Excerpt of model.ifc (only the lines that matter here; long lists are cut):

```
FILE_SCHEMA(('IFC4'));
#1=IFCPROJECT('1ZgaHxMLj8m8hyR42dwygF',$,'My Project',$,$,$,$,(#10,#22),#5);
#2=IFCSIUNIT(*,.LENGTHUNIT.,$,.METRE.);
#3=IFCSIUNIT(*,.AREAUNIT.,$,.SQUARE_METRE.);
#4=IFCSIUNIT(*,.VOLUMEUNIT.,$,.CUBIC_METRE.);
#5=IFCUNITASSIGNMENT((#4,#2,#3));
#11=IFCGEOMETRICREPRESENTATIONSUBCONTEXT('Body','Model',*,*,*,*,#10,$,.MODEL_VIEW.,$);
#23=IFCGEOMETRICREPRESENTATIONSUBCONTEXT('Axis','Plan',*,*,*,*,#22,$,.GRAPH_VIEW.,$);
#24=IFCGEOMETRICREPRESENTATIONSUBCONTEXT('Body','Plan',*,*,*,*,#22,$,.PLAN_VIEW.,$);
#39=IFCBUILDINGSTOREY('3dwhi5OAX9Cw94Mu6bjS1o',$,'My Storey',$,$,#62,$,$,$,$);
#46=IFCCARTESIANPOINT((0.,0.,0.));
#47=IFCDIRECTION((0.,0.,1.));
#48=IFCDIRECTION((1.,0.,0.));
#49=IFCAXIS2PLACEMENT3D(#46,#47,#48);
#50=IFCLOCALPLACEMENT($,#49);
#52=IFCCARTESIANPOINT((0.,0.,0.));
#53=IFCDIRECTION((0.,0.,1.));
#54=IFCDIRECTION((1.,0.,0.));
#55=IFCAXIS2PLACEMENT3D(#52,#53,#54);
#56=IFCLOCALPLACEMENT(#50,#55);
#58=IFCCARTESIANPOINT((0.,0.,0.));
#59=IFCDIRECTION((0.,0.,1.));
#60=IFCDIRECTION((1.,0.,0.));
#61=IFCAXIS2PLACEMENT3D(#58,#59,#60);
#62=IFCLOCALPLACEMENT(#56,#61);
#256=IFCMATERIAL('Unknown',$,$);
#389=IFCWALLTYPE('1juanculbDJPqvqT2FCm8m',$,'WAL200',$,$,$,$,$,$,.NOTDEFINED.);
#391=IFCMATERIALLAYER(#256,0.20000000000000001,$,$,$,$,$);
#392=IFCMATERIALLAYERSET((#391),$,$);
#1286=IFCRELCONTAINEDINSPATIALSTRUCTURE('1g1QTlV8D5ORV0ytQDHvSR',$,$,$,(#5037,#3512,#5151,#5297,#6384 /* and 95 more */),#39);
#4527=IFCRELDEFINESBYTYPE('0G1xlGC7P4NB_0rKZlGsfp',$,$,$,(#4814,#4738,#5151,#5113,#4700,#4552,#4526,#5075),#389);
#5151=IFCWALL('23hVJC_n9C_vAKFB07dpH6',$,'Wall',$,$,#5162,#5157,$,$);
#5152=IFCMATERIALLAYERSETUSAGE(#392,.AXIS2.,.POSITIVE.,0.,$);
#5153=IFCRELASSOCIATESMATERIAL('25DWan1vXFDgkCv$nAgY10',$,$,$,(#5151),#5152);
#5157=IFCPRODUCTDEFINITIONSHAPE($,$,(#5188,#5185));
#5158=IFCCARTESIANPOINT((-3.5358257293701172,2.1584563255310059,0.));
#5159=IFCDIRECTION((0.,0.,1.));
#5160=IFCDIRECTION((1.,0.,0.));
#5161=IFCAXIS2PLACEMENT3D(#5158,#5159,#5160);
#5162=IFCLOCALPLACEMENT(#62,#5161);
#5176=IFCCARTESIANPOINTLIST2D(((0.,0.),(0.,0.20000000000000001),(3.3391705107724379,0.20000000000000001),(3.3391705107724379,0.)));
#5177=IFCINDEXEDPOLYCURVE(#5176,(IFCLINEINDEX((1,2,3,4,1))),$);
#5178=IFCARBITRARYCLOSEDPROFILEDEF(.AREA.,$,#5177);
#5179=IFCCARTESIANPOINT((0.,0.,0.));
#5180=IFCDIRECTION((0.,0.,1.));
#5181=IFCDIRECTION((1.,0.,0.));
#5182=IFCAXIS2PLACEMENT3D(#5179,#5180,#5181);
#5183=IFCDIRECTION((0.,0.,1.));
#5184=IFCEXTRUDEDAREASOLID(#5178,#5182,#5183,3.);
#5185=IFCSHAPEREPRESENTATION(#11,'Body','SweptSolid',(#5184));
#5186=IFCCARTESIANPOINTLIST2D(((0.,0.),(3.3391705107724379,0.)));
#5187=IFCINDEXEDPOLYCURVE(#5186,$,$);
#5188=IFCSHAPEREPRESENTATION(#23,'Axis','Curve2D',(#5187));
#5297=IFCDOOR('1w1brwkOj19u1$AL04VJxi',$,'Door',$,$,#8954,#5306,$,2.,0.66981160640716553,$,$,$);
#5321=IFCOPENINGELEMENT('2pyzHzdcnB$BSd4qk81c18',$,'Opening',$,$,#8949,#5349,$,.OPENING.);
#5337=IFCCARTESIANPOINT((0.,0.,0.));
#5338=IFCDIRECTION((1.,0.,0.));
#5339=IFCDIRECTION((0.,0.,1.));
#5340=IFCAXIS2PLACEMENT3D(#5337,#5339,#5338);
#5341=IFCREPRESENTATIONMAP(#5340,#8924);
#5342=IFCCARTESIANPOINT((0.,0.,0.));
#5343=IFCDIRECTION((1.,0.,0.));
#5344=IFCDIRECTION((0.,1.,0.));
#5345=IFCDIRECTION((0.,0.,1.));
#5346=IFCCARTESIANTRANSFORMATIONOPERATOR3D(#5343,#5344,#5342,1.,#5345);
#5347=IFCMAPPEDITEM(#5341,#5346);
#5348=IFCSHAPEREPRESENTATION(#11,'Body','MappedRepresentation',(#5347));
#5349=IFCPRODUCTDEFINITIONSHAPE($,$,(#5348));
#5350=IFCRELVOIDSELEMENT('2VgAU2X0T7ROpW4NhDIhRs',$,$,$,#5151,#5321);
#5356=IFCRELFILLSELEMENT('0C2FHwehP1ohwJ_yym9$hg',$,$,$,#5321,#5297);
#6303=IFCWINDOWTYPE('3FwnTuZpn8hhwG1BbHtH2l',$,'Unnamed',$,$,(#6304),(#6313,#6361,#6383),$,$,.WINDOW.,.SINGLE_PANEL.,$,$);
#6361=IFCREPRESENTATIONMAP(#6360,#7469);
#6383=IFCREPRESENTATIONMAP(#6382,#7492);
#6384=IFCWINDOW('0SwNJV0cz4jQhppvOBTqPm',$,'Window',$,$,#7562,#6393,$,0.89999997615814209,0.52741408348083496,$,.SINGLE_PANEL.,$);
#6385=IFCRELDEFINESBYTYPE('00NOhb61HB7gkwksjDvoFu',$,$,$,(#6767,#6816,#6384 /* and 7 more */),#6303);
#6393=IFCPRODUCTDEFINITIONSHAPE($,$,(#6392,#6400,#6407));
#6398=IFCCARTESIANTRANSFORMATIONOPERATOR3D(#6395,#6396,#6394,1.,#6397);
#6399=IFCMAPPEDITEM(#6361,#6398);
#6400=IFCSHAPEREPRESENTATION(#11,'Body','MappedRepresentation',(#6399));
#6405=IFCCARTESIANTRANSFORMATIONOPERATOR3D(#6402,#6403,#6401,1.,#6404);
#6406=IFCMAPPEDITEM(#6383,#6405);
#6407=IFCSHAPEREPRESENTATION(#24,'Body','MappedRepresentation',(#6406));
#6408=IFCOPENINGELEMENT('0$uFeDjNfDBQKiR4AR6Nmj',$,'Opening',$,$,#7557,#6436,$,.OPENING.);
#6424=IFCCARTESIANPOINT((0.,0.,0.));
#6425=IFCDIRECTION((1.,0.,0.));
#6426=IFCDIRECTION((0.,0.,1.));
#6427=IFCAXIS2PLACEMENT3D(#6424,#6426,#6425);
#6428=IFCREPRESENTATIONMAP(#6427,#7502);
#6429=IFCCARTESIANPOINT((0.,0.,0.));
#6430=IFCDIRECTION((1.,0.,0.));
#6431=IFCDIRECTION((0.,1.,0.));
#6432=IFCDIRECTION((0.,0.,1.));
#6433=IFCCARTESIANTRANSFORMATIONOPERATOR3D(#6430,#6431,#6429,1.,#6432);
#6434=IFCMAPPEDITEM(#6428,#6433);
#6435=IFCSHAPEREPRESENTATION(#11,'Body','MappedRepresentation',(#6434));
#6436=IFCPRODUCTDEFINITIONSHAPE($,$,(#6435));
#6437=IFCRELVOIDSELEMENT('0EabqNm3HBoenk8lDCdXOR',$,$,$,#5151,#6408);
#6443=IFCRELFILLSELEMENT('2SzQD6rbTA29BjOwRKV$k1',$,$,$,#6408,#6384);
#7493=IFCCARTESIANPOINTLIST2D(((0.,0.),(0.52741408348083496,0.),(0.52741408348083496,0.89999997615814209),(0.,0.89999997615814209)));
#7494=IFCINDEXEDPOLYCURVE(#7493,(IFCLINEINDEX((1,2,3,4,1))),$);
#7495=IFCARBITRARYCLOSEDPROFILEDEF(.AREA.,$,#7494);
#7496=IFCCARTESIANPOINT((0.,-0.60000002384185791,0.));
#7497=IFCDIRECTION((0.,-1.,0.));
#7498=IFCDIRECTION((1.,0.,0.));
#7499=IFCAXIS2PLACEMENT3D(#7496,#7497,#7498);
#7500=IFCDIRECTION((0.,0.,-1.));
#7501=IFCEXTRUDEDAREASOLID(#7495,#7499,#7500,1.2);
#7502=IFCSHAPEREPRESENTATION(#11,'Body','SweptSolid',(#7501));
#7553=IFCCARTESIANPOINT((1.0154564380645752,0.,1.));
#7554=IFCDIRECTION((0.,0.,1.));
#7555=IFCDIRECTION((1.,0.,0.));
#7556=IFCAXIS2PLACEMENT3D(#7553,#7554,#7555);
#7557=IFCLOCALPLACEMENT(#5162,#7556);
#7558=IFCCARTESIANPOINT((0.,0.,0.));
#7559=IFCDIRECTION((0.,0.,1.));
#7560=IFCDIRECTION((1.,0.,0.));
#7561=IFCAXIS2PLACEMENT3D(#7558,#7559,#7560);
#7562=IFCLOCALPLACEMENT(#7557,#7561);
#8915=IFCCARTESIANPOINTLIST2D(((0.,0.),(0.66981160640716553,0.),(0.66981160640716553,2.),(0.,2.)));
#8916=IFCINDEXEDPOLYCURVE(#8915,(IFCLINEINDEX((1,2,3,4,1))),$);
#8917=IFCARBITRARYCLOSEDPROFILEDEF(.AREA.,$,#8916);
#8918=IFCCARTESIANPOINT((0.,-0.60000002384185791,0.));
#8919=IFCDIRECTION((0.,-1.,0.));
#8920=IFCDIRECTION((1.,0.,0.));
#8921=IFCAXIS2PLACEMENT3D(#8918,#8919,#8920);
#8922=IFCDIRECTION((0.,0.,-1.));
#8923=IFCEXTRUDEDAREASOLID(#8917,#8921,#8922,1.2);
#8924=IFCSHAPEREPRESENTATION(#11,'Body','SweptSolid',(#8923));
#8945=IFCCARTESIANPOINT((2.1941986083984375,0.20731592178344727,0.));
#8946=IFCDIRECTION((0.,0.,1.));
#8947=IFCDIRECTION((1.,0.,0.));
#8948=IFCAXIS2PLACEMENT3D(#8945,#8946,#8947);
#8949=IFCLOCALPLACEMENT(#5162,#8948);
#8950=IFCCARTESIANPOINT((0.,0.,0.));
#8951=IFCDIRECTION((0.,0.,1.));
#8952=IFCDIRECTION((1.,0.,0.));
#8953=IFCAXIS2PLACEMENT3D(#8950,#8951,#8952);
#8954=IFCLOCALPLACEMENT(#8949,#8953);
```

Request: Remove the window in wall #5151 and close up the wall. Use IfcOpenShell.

```python
import ifcopenshell
import ifcopenshell.api.feature
import ifcopenshell.api.root
import ifcopenshell.geom
import ifcopenshell.util.shape

model = ifcopenshell.open("model.ifc")
settings = ifcopenshell.geom.settings()


def volume(element):
    """Net volume in cubic metres, openings subtracted."""
    shape = ifcopenshell.geom.create_shape(settings, element)
    return ifcopenshell.util.shape.get_volume(shape.geometry)


window = model.by_guid("0SwNJV0cz4jQhppvOBTqPm")
opening = window.FillsVoids[0].RelatingOpeningElement
wall = opening.VoidsElements[0].RelatingBuildingElement
before = volume(wall)

ifcopenshell.api.root.remove_product(model, product=window)
ifcopenshell.api.feature.remove_feature(model, feature=opening)

after = volume(wall)

print(f"wall volume {before:.3f} -> {after:.3f} m3")

model.write("model_updated.ifc")
```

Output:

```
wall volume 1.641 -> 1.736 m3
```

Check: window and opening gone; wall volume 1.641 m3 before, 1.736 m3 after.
